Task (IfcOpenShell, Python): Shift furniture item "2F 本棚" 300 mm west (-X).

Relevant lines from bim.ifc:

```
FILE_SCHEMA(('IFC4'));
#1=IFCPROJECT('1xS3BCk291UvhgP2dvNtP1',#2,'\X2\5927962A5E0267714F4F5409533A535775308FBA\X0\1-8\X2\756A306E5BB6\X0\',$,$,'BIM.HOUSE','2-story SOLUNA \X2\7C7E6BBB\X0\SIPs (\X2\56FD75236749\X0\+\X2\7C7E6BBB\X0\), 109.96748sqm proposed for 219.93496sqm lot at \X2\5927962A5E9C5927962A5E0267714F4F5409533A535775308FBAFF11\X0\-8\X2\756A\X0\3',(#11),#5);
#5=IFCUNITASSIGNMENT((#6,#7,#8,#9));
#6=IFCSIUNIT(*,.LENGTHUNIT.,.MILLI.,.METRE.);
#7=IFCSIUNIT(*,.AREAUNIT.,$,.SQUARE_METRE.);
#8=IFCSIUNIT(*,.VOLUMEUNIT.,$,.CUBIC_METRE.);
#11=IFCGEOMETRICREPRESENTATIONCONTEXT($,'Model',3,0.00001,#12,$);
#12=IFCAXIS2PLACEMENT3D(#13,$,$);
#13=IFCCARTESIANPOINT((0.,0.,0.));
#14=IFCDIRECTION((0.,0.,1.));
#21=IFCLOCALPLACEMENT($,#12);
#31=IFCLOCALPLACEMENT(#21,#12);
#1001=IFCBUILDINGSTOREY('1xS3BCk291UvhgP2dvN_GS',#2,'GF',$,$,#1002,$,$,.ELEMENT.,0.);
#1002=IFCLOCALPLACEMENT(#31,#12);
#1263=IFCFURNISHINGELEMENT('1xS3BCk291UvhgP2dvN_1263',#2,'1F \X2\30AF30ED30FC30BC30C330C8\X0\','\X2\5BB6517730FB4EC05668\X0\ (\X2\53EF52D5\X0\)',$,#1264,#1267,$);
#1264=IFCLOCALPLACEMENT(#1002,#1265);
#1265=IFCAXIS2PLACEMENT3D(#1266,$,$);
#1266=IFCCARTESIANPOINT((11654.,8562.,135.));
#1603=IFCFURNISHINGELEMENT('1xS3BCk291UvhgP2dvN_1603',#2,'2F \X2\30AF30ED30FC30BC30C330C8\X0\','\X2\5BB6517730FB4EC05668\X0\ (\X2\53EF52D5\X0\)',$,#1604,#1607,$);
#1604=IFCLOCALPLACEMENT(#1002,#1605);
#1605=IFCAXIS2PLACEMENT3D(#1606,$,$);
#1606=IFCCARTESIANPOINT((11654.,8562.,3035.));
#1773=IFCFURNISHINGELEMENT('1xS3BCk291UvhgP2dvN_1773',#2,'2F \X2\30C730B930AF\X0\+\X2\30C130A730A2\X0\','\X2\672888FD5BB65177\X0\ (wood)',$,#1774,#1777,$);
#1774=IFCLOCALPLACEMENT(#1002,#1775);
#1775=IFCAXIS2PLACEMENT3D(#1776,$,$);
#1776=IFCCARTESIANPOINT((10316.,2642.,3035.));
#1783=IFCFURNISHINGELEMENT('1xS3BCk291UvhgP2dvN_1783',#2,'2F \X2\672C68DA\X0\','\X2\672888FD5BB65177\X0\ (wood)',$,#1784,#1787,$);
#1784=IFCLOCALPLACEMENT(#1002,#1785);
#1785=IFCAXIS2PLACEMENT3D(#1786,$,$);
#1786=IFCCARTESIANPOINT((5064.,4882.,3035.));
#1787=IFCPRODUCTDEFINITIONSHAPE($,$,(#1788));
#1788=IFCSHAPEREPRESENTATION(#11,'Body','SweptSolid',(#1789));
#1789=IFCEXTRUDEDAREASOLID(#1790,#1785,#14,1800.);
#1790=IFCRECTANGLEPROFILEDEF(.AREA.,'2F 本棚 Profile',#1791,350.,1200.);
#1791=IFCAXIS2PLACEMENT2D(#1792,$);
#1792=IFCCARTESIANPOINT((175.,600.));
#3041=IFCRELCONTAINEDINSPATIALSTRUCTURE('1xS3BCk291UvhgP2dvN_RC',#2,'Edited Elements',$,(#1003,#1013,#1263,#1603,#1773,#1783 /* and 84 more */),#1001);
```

```python
import ifcopenshell
import ifcopenshell.api.geometry
import ifcopenshell.util.placement
import ifcopenshell.util.unit

model = ifcopenshell.open("bim.ifc")
unit_scale = ifcopenshell.util.unit.calculate_unit_scale(model)

item = model.by_guid("1xS3BCk291UvhgP2dvN_1783")
matrix = ifcopenshell.util.placement.get_local_placement(item.ObjectPlacement)
matrix[0, 3] -= 0.3 / unit_scale
ifcopenshell.api.geometry.edit_object_placement(model, product=item, matrix=matrix, is_si=False)

print(ifcopenshell.util.placement.get_local_placement(item.ObjectPlacement).round(3) + 0.0)

model.write("bim_v2.ifc")
```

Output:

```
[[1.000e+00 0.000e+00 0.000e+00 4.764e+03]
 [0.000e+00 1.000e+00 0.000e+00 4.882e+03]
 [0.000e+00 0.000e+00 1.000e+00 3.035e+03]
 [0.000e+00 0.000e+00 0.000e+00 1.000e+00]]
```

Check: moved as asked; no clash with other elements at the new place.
